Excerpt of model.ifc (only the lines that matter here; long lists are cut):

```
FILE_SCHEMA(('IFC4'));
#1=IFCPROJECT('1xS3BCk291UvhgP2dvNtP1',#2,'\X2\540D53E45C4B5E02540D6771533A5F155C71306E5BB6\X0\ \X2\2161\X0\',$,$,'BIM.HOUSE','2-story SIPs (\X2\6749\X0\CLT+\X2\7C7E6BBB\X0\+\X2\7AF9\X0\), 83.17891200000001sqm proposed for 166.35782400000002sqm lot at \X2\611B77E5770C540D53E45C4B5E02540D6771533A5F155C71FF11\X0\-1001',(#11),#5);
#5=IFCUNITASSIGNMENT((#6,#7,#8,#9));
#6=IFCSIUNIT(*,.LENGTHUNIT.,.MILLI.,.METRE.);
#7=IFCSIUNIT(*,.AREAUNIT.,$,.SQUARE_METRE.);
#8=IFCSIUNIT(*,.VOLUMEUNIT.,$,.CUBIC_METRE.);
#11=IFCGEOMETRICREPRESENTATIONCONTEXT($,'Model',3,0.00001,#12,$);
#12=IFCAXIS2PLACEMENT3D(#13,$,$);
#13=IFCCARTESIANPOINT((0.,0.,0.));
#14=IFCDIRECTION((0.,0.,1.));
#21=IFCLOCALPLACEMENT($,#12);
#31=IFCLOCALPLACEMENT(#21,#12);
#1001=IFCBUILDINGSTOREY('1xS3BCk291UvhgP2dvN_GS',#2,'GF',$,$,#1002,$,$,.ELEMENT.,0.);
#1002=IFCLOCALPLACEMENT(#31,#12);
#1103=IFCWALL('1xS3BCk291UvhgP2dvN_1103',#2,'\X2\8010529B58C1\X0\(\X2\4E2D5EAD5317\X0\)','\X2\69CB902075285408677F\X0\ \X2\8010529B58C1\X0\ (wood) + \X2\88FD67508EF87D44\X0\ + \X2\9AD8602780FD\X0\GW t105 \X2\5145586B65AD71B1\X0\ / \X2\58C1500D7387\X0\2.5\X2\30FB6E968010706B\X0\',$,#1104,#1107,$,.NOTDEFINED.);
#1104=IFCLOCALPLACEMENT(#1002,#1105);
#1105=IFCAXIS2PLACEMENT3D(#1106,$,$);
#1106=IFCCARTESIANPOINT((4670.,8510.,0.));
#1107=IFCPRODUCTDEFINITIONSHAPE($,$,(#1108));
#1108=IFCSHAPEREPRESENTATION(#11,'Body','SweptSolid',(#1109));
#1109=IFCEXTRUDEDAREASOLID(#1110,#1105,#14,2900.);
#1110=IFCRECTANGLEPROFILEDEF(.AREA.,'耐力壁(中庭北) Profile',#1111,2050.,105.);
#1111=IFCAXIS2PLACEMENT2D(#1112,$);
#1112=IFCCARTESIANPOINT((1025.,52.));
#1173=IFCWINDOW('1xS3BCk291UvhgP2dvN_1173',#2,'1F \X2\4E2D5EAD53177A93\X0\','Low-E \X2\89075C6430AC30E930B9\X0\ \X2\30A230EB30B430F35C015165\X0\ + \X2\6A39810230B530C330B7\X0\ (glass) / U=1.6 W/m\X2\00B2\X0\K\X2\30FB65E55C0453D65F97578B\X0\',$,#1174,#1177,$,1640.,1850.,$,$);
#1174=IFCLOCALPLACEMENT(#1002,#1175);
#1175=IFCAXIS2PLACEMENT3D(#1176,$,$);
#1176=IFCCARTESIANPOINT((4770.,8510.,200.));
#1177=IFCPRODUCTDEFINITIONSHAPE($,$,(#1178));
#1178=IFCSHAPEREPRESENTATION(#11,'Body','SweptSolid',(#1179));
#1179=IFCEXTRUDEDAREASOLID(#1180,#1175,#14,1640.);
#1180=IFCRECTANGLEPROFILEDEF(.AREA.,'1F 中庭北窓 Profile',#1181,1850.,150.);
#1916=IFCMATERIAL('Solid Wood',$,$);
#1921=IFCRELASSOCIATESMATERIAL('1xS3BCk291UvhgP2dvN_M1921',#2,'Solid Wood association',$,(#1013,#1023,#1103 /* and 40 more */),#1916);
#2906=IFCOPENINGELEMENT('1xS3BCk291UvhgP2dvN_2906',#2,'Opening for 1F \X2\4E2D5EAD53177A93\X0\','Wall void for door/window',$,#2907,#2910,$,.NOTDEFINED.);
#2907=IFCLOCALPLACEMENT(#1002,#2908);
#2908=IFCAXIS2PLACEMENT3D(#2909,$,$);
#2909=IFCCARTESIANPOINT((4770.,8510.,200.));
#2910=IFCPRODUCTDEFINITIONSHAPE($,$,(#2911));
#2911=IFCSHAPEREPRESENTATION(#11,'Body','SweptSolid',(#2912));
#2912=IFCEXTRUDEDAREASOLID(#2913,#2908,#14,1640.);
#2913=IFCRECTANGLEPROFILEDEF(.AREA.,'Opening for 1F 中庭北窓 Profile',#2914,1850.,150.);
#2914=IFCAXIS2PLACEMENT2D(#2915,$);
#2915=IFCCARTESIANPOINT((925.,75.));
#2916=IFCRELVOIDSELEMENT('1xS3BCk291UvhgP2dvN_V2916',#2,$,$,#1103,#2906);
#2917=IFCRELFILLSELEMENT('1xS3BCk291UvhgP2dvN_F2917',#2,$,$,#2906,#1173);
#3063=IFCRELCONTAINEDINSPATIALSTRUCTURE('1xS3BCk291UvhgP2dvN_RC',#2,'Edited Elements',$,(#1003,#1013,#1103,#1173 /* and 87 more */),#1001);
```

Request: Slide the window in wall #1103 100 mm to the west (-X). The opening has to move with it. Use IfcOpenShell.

```python
import ifcopenshell
import ifcopenshell.api.geometry
import ifcopenshell.util.placement
import ifcopenshell.util.unit

model = ifcopenshell.open("model.ifc")
unit_scale = ifcopenshell.util.unit.calculate_unit_scale(model)

window = model.by_id(1173)
opening = window.FillsVoids[0].RelatingOpeningElement
wall = opening.VoidsElements[0].RelatingBuildingElement

wall_matrix = ifcopenshell.util.placement.get_local_placement(wall.ObjectPlacement)
shift = wall_matrix[:3, 0] * -0.1 / unit_scale
before = ifcopenshell.util.placement.get_local_placement(window.ObjectPlacement)[:3, 3].copy()

# The window is not placed relative to its opening, so move both.
for product in (opening, window):
    matrix = ifcopenshell.util.placement.get_local_placement(product.ObjectPlacement)
    matrix[:3, 3] += shift
    ifcopenshell.api.geometry.edit_object_placement(model, product=product, matrix=matrix, is_si=False)

after = ifcopenshell.util.placement.get_local_placement(window.ObjectPlacement)[:3, 3]
print("window moved by", (after - before).round(3) + 0.0)

model.write("model-out.ifc")
```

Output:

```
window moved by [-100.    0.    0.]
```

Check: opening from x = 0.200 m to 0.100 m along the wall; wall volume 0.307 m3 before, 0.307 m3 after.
